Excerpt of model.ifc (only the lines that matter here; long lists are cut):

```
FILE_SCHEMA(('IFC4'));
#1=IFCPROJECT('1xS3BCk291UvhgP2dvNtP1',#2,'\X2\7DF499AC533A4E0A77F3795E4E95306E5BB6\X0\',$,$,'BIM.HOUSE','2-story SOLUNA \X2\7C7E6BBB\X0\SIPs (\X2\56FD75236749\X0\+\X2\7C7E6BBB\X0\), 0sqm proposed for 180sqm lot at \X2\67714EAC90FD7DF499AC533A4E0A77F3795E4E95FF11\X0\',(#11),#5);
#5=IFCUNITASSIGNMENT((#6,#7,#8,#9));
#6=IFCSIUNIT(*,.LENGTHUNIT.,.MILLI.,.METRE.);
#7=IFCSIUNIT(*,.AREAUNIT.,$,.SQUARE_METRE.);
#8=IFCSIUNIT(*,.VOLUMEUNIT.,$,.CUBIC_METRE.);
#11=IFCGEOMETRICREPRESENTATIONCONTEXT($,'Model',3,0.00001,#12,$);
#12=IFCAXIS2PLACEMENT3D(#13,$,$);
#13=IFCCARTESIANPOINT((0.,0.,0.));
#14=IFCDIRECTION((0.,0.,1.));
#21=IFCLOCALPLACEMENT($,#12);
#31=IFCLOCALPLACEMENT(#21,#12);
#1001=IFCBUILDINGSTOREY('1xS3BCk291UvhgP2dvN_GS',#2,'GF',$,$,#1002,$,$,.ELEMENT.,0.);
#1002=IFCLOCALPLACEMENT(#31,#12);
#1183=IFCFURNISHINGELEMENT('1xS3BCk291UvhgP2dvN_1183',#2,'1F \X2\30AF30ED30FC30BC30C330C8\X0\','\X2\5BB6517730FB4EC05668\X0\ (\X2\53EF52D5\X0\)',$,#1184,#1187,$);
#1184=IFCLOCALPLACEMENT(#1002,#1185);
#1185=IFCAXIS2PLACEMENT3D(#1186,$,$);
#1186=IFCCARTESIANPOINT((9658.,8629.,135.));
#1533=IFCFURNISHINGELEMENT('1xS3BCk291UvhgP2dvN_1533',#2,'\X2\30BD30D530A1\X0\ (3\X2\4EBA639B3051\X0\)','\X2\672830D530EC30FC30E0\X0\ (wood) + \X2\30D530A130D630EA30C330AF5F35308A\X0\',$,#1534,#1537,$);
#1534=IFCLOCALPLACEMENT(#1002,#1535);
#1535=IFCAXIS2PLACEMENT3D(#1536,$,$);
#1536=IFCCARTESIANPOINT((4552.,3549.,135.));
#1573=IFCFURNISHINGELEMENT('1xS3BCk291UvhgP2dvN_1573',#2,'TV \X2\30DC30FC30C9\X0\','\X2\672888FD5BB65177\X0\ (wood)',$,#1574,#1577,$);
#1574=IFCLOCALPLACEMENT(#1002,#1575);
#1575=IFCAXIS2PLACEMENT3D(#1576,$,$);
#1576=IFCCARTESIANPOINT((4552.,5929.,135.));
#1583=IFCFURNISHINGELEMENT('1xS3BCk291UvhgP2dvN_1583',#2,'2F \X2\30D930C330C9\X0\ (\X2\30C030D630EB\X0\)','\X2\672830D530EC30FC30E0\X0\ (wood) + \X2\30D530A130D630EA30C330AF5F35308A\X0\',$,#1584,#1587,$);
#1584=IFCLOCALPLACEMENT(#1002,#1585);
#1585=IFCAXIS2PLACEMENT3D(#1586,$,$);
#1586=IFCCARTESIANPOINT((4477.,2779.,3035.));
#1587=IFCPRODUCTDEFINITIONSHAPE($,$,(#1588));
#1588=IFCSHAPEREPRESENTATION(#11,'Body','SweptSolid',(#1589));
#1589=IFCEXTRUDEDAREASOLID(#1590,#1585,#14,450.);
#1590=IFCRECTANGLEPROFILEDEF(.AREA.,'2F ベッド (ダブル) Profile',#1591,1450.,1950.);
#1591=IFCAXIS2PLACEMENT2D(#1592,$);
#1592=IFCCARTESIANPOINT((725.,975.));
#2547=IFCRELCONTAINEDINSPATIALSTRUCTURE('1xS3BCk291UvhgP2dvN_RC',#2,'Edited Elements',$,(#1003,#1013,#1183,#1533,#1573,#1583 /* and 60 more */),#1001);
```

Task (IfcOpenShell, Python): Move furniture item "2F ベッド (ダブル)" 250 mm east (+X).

```python
import ifcopenshell
import ifcopenshell.api.geometry
import ifcopenshell.util.placement
import ifcopenshell.util.unit

model = ifcopenshell.open("model.ifc")
unit_scale = ifcopenshell.util.unit.calculate_unit_scale(model)

item = model.by_id(1583)
matrix = ifcopenshell.util.placement.get_local_placement(item.ObjectPlacement)
matrix[0, 3] += 0.25 / unit_scale
ifcopenshell.api.geometry.edit_object_placement(model, product=item, matrix=matrix, is_si=False)

print(ifcopenshell.util.placement.get_local_placement(item.ObjectPlacement).round(3) + 0.0)

model.write("model_rev.ifc")
```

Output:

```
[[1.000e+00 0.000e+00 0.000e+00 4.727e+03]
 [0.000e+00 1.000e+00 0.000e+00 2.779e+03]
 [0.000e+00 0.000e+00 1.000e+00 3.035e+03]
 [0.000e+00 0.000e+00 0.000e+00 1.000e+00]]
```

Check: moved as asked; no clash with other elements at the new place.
